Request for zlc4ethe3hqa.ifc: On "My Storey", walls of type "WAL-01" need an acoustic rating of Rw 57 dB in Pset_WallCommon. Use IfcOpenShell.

First a look at what the model holds.

```python
import ifcopenshell
import ifcopenshell.util.element

model = ifcopenshell.open("zlc4ethe3hqa.ifc")
print(model.schema)
storey = next(s for s in model.by_type("IfcBuildingStorey") if s.Name == "My Storey")
walls = [e for e in ifcopenshell.util.element.get_decomposition(storey) if e.is_a("IfcWall")]
seen = {}
for e in walls:
    element_type = ifcopenshell.util.element.get_type(e)
    key = (element_type.Name if element_type != e and element_type else None, ifcopenshell.util.element.get_pset(e, "Pset_WallCommon", "AcousticRating"))
    seen[key] = seen.get(key, 0) + 1
for (name, value), count in sorted(seen.items(), key=str):
    print(count, "x", name, "|", value)
```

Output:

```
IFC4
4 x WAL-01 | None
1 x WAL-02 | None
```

```python
import ifcopenshell
import ifcopenshell.api.pset
import ifcopenshell.util.element

model = ifcopenshell.open("zlc4ethe3hqa.ifc")

storey = next(s for s in model.by_type("IfcBuildingStorey") if s.Name == "My Storey")
walls = [e for e in ifcopenshell.util.element.get_decomposition(storey) if e.is_a("IfcWall")]

count = 0
for e in walls:
    element_type = ifcopenshell.util.element.get_type(e)
    if element_type in (None, e) or element_type.Name != "WAL-01":
        continue
    # add_pset returns the element's existing set when there is one.
    pset = ifcopenshell.api.pset.add_pset(model, product=e, name="Pset_WallCommon")
    ifcopenshell.api.pset.edit_pset(model, pset=pset, properties={"AcousticRating": "Rw 57 dB"})
    count += 1

print(count, "walls updated")

model.write("zlc4ethe3hqa_v2.ifc")
```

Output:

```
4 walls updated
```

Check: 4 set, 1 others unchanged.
